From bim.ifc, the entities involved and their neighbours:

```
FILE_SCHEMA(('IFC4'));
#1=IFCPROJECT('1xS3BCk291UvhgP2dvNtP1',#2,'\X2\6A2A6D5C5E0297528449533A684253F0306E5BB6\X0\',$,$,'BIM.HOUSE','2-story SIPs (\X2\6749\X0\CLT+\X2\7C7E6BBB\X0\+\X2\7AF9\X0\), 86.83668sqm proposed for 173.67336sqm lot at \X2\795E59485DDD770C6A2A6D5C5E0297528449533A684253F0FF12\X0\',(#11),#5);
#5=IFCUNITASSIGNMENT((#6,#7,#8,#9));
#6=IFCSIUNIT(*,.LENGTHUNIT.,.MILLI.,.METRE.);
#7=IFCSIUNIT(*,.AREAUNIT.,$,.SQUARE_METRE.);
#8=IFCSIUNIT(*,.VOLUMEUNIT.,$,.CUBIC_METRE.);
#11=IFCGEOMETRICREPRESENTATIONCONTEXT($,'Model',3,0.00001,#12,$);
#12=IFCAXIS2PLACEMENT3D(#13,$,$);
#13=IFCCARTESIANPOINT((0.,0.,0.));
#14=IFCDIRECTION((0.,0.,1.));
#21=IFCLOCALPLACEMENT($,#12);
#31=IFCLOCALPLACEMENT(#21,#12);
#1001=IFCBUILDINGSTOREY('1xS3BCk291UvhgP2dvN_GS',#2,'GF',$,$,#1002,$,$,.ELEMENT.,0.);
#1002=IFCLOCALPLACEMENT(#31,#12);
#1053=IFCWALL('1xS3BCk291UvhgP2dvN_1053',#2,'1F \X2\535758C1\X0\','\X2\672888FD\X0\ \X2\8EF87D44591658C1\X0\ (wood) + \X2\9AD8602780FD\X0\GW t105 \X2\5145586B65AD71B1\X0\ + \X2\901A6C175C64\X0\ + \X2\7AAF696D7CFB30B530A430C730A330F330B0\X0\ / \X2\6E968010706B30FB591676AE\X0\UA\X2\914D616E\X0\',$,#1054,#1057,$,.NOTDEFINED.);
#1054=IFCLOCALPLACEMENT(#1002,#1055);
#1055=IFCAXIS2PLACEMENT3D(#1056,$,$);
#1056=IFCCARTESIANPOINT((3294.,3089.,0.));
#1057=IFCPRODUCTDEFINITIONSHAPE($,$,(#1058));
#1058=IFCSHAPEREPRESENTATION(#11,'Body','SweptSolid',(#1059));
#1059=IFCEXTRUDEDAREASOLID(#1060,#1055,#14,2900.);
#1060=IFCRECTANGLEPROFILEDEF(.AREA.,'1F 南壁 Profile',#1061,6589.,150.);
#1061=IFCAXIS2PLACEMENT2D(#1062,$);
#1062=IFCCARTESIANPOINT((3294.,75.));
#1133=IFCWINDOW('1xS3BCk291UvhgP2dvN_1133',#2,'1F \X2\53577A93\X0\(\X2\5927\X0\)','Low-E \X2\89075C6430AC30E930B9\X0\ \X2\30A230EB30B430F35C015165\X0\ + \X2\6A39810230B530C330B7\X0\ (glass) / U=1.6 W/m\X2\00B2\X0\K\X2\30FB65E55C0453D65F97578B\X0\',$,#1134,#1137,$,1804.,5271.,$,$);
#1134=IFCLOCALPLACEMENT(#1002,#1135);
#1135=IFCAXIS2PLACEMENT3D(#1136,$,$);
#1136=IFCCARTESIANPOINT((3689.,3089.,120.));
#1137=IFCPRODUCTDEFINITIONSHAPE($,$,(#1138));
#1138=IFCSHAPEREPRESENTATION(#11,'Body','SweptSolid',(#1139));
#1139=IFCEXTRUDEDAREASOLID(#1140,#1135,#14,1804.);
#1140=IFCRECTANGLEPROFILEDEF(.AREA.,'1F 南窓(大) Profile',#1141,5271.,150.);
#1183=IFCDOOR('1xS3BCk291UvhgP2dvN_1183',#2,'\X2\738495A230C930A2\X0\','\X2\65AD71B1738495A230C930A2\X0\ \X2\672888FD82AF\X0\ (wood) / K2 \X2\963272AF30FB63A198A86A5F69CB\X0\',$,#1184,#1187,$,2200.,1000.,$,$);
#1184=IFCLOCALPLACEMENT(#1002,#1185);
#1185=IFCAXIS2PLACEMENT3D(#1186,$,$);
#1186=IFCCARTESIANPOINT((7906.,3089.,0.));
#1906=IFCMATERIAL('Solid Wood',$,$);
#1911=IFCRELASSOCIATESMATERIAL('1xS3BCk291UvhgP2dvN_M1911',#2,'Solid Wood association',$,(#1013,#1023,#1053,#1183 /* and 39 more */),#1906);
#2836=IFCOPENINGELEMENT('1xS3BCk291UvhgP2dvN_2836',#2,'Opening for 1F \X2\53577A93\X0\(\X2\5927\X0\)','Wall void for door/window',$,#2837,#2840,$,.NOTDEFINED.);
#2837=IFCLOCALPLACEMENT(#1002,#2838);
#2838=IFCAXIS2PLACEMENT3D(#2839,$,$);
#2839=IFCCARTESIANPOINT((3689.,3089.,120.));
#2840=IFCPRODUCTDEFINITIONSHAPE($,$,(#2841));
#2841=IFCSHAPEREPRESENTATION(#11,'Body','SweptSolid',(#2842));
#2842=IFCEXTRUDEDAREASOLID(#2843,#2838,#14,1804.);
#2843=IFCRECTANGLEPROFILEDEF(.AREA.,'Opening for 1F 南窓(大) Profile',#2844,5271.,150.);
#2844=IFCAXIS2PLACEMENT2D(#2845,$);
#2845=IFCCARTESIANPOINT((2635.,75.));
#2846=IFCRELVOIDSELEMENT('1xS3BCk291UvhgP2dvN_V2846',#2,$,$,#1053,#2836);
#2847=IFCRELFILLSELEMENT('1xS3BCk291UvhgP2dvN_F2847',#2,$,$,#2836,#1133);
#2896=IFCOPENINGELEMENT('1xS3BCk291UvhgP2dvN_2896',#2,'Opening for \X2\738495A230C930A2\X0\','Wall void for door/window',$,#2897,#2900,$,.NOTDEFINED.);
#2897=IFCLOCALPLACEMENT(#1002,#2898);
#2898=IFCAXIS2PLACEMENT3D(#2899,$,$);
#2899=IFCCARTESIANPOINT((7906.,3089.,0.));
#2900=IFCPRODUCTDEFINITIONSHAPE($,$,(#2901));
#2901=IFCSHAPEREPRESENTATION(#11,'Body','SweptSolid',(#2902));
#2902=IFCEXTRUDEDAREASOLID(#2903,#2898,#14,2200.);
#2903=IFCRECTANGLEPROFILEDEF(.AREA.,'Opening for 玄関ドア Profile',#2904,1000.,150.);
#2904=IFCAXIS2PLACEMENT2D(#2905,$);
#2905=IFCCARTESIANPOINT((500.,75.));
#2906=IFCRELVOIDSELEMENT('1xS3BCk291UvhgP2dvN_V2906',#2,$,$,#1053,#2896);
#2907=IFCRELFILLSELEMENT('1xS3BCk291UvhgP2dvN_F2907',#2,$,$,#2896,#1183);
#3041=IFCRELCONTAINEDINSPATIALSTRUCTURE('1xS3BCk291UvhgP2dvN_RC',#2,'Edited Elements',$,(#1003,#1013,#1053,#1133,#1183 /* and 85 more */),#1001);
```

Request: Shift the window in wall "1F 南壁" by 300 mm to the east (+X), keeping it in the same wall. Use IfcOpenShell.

```python
import ifcopenshell
import ifcopenshell.api.geometry
import ifcopenshell.util.placement

model = ifcopenshell.open("bim.ifc")

window = model.by_id(1133)
opening = window.FillsVoids[0].RelatingOpeningElement
wall = opening.VoidsElements[0].RelatingBuildingElement

wall_matrix = ifcopenshell.util.placement.get_local_placement(wall.ObjectPlacement)
shift = wall_matrix[:3, 0] * 300.0
before = ifcopenshell.util.placement.get_local_placement(window.ObjectPlacement)[:3, 3].copy()

# The window is not placed relative to its opening, so move both.
for product in (opening, window):
    matrix = ifcopenshell.util.placement.get_local_placement(product.ObjectPlacement)
    matrix[:3, 3] += shift
    ifcopenshell.api.geometry.edit_object_placement(model, product=product, matrix=matrix, is_si=False)

after = ifcopenshell.util.placement.get_local_placement(window.ObjectPlacement)[:3, 3]
print("window moved by", (after - before).round(3) + 0.0)

model.write("bim-out.ifc")
```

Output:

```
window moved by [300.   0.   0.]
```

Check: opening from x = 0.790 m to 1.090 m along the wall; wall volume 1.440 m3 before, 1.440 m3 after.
